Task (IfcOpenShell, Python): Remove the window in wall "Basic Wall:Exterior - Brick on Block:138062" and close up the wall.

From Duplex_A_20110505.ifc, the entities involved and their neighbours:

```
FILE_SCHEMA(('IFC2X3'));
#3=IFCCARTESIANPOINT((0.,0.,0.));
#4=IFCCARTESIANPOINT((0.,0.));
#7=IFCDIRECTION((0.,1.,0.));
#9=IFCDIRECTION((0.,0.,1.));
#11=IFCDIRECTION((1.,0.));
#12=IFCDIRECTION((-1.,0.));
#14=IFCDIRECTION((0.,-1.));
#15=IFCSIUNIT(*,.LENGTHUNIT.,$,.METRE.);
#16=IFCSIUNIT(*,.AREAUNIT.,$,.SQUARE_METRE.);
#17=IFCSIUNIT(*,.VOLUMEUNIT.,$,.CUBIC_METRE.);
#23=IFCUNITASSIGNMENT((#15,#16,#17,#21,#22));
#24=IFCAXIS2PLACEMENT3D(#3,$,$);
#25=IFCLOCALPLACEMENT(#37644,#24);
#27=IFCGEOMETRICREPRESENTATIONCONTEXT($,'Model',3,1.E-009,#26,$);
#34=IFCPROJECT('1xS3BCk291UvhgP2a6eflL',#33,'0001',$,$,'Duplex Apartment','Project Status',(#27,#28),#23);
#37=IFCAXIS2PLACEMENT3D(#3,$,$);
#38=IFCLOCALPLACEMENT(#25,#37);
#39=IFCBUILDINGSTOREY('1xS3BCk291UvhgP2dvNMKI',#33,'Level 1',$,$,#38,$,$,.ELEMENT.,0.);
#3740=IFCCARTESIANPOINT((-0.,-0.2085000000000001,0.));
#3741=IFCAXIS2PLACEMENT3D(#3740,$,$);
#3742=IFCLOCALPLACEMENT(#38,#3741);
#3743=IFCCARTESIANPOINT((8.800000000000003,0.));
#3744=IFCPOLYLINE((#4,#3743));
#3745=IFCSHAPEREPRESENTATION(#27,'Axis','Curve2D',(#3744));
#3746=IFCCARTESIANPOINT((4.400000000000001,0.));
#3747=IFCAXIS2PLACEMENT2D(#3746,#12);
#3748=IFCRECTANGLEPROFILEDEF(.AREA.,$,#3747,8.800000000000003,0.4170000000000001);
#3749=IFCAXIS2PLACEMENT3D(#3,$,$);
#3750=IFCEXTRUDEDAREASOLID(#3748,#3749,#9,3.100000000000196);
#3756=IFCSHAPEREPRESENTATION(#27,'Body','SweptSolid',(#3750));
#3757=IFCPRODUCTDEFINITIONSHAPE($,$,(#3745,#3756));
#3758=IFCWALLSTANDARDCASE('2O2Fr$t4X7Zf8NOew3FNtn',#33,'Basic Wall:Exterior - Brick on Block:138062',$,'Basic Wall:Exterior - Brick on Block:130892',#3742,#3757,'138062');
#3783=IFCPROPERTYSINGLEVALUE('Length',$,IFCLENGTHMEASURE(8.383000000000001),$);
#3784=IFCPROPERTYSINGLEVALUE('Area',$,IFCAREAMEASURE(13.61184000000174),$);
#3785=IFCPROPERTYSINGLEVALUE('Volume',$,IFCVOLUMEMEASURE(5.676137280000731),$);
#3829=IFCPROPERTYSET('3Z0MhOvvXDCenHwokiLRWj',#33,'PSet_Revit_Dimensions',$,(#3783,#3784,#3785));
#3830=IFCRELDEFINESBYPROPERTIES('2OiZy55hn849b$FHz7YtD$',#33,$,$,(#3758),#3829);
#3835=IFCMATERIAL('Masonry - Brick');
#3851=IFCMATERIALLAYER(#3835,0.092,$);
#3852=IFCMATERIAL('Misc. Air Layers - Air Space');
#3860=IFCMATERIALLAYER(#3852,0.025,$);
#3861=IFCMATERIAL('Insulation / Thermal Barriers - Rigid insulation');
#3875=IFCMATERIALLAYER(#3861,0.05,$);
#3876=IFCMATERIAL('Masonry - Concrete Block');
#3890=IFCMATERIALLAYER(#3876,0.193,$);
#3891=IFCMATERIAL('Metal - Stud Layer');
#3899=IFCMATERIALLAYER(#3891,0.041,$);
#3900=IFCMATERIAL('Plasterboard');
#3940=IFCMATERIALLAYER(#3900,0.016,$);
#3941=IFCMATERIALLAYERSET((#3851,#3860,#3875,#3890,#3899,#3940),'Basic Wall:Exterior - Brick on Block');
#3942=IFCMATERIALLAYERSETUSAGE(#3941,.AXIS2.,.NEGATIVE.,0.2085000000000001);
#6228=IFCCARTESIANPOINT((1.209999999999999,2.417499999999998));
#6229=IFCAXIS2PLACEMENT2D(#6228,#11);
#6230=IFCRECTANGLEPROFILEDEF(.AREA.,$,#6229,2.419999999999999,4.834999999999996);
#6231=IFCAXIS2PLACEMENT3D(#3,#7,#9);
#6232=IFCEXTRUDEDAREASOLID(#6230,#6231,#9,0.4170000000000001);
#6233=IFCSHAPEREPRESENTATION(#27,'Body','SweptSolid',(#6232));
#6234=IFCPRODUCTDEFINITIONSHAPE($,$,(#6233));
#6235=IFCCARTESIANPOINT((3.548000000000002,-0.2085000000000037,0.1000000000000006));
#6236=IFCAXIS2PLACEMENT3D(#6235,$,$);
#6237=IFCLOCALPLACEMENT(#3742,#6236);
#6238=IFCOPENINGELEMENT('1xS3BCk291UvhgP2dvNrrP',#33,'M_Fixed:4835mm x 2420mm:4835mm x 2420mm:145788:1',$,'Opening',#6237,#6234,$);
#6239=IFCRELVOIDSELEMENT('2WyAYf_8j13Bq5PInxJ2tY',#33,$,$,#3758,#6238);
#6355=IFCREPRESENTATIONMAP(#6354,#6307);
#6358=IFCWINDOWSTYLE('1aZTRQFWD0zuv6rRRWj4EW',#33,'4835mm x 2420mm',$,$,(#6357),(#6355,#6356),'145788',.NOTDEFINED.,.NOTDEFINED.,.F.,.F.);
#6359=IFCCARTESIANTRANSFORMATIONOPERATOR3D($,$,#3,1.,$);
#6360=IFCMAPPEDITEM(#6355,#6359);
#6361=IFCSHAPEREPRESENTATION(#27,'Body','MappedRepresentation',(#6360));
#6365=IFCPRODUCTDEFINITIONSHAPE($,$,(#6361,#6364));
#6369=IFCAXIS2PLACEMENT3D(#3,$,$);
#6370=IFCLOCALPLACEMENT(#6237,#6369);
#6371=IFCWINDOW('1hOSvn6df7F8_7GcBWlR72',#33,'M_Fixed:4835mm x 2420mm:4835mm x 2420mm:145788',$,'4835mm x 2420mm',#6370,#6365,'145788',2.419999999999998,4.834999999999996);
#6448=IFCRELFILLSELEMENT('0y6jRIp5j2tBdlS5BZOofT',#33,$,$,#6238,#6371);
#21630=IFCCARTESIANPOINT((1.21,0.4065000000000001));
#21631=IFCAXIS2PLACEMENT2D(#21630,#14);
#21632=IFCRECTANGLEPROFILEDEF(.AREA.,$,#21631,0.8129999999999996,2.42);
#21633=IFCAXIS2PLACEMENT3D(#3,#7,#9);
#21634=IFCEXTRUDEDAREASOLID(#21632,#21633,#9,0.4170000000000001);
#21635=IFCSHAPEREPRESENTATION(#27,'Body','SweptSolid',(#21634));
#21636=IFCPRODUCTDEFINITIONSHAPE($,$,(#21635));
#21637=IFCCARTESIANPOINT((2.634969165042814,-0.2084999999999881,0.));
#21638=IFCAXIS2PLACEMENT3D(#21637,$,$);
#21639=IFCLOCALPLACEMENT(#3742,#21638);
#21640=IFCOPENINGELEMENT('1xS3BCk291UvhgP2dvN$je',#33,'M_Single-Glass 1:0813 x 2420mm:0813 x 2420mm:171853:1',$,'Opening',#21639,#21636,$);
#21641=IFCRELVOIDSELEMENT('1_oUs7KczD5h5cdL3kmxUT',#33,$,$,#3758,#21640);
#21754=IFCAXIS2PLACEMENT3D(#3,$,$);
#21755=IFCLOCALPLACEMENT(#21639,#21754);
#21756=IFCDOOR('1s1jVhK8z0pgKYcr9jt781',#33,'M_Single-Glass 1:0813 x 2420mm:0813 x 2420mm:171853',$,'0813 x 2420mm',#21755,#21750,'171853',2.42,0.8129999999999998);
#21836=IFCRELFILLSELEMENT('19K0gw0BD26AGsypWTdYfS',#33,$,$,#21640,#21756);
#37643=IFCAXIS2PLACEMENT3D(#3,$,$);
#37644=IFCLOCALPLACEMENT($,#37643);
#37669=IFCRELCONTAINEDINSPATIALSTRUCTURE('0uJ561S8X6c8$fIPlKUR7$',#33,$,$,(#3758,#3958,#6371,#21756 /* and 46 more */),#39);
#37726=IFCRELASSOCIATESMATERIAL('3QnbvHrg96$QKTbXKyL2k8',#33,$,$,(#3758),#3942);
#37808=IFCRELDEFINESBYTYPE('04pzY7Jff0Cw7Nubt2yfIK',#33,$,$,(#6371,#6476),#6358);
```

```python
import ifcopenshell
import ifcopenshell.api.feature
import ifcopenshell.api.pset
import ifcopenshell.api.root
import ifcopenshell.geom
import ifcopenshell.util.element
import ifcopenshell.util.shape
import ifcopenshell.util.unit

model = ifcopenshell.open("Duplex_A_20110505.ifc")
area_scale = ifcopenshell.util.unit.calculate_unit_scale(model, "AREAUNIT")
volume_scale = ifcopenshell.util.unit.calculate_unit_scale(model, "VOLUMEUNIT")
settings = ifcopenshell.geom.settings()


def volume(element):
    """Net volume in cubic metres, openings subtracted."""
    shape = ifcopenshell.geom.create_shape(settings, element)
    return ifcopenshell.util.shape.get_volume(shape.geometry)


window = model.by_id(6371)
opening = window.FillsVoids[0].RelatingOpeningElement
wall = opening.VoidsElements[0].RelatingBuildingElement
before = volume(wall)

ifcopenshell.api.root.remove_product(model, product=window)
ifcopenshell.api.feature.remove_feature(model, feature=opening)

after = volume(wall)
thickness = 0.417  # wall thickness in metres

# Update the wall's stored quantities.
pset = model.by_id(ifcopenshell.util.element.get_pset(wall, "PSet_Revit_Dimensions", should_inherit=False)["id"])
ifcopenshell.api.pset.edit_pset(model, pset=pset, properties={
    "Area": model.create_entity("IfcAreaMeasure", after / thickness / area_scale),
    "Volume": model.create_entity("IfcVolumeMeasure", after / volume_scale),
})

print(f"wall volume {before:.3f} -> {after:.3f} m3")

model.write("Duplex_A_20110505_edited.ifc")
```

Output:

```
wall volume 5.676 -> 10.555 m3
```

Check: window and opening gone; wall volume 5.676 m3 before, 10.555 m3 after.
